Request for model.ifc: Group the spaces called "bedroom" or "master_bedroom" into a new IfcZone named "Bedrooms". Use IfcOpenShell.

First a look at what the model holds.

```python
import ifcopenshell

model = ifcopenshell.open("model.ifc")
print(model.schema)
seen = {}
for space in model.by_type("IfcSpace"):
    seen[space.LongName] = seen.get(space.LongName, 0) + 1
for name, count in sorted(seen.items(), key=str):
    print(count, "x", name)
print("zones:", [z.Name for z in model.by_type("IfcZone")][:20])
```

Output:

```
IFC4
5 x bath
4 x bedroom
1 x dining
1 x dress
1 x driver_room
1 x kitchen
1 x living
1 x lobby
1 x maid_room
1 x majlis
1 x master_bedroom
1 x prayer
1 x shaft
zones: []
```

```python
import ifcopenshell
import ifcopenshell.api.group
import ifcopenshell.api.root

model = ifcopenshell.open("model.ifc")

names = {"bedroom", "master_bedroom"}
spaces = [s for s in model.by_type("IfcSpace") if s.LongName in names]

zone = ifcopenshell.api.root.create_entity(model, ifc_class="IfcZone", name="Bedrooms")
ifcopenshell.api.group.assign_group(model, products=spaces, group=zone)
print(len(spaces), "spaces in", zone.Name)

model.write("model-out.ifc")
```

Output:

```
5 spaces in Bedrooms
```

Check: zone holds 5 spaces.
